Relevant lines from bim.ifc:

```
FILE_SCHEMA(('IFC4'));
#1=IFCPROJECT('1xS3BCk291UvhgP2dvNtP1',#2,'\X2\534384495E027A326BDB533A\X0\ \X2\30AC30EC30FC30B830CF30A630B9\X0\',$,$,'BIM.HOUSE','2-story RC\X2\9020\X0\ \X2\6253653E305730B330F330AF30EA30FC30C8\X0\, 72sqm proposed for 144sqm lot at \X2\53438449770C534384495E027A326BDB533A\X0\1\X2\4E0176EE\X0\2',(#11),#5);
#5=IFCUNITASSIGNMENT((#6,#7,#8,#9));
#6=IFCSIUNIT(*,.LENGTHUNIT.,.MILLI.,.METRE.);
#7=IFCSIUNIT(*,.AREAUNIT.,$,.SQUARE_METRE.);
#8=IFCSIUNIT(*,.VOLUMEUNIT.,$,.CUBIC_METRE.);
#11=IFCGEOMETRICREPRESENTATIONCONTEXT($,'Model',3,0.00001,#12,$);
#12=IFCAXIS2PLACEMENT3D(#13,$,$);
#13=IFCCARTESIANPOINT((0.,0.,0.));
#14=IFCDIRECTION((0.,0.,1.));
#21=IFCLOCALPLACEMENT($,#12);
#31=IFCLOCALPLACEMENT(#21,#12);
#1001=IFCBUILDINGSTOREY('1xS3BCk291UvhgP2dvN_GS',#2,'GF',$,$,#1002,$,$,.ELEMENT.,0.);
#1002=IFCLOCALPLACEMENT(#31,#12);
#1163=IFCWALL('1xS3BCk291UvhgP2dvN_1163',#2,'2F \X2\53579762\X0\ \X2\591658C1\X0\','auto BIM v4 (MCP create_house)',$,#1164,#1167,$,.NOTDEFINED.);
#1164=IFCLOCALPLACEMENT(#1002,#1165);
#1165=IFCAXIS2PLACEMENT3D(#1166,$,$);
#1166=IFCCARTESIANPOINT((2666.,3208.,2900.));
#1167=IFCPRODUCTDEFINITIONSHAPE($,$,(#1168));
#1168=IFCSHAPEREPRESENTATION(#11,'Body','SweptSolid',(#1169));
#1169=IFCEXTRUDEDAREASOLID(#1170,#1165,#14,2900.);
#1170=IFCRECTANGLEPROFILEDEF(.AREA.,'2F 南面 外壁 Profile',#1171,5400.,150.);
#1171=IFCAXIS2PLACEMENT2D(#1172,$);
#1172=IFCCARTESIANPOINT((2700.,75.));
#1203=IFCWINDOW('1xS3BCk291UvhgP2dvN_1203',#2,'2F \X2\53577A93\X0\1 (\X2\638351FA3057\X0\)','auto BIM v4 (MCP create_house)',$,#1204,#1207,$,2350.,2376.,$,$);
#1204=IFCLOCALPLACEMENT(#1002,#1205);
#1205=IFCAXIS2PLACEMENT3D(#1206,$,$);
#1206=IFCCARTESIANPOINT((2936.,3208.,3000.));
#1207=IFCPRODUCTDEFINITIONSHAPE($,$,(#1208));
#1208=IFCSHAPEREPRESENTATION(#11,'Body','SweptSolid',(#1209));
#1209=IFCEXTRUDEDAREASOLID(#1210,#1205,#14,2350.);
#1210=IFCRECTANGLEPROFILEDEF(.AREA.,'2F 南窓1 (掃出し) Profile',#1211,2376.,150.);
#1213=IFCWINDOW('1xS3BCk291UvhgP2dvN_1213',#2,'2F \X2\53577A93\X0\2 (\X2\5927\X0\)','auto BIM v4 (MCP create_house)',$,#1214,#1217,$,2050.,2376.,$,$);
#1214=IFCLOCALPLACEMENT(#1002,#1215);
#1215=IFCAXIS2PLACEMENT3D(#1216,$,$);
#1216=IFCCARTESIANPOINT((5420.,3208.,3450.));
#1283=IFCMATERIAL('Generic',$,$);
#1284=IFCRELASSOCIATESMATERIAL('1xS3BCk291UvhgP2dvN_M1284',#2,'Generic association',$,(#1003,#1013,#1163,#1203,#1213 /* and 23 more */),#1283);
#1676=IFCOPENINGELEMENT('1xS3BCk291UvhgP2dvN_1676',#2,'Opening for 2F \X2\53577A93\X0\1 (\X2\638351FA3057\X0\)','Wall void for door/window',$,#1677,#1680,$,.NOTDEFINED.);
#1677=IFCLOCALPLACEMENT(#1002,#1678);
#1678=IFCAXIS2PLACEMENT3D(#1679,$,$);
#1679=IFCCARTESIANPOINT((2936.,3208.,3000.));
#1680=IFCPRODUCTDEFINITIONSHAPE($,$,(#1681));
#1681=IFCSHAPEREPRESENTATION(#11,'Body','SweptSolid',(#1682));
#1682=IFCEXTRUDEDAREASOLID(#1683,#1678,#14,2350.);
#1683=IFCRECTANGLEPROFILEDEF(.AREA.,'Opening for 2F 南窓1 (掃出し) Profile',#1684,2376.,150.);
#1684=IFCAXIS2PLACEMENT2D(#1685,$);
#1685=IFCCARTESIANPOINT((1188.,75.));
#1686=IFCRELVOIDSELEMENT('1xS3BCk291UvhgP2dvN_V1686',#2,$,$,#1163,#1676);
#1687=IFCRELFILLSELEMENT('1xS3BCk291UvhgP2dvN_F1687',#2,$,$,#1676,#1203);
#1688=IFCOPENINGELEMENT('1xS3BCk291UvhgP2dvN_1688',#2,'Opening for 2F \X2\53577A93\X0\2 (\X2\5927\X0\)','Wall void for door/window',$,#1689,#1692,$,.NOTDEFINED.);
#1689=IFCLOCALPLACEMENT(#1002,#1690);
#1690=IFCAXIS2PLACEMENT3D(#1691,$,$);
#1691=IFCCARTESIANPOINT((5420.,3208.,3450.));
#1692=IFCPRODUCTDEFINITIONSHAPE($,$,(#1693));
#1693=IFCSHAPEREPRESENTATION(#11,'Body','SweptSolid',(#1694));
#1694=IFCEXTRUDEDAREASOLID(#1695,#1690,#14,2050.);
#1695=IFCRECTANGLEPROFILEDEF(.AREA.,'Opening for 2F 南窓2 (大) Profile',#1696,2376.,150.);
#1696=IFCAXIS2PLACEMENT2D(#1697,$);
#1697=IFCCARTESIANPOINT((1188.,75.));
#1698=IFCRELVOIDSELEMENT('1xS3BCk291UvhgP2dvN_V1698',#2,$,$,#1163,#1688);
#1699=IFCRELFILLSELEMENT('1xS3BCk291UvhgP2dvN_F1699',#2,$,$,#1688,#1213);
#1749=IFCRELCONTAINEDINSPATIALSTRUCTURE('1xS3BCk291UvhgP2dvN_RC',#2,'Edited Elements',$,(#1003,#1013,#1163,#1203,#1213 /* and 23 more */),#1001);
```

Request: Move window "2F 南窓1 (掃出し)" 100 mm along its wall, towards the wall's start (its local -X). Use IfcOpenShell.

```python
import ifcopenshell
import ifcopenshell.api.geometry
import ifcopenshell.util.placement
import ifcopenshell.util.unit

model = ifcopenshell.open("bim.ifc")
unit_scale = ifcopenshell.util.unit.calculate_unit_scale(model)

window = model.by_id(1203)
opening = window.FillsVoids[0].RelatingOpeningElement
wall = opening.VoidsElements[0].RelatingBuildingElement

wall_matrix = ifcopenshell.util.placement.get_local_placement(wall.ObjectPlacement)
shift = wall_matrix[:3, 0] * -0.1 / unit_scale
before = ifcopenshell.util.placement.get_local_placement(window.ObjectPlacement)[:3, 3].copy()

# The window is not placed relative to its opening, so move both.
for product in (opening, window):
    matrix = ifcopenshell.util.placement.get_local_placement(product.ObjectPlacement)
    matrix[:3, 3] += shift
    ifcopenshell.api.geometry.edit_object_placement(model, product=product, matrix=matrix, is_si=False)

after = ifcopenshell.util.placement.get_local_placement(window.ObjectPlacement)[:3, 3]
print("window moved by", (after - before).round(3) + 0.0)

model.write("bim_edited.ifc")
```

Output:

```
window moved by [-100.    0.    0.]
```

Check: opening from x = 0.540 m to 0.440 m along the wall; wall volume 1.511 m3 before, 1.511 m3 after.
